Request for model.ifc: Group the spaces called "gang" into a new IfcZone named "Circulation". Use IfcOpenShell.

First a look at what the model holds.

```python
import ifcopenshell

model = ifcopenshell.open("model.ifc")
print(model.schema)
seen = {}
for space in model.by_type("IfcSpace"):
    seen[space.LongName] = seen.get(space.LongName, 0) + 1
for name, count in sorted(seen.items(), key=str):
    print(count, "x", name)
print("zones:", [z.Name for z in model.by_type("IfcZone")][:20])
```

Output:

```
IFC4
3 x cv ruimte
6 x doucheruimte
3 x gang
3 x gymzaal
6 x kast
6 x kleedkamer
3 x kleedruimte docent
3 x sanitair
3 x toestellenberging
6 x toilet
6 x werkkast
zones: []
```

```python
import ifcopenshell
import ifcopenshell.api.group
import ifcopenshell.api.root

model = ifcopenshell.open("model.ifc")

names = {"gang"}
spaces = [s for s in model.by_type("IfcSpace") if s.LongName in names]

zone = ifcopenshell.api.root.create_entity(model, ifc_class="IfcZone", name="Circulation")
ifcopenshell.api.group.assign_group(model, products=spaces, group=zone)
print(len(spaces), "spaces in", zone.Name)

model.write("model_edited.ifc")
```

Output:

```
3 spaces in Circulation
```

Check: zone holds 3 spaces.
